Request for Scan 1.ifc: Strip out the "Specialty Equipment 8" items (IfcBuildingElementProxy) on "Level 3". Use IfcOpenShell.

First a look at what the model holds.

```python
import ifcopenshell
import ifcopenshell.util.element

model = ifcopenshell.open("Scan 1.ifc")
print(model.schema)
storey = next(s for s in model.by_type("IfcBuildingStorey") if s.Name == "Level 3")
proxies = [e for e in ifcopenshell.util.element.get_decomposition(storey) if e.is_a("IfcBuildingElementProxy")]
seen = {}
for e in proxies:
    element_type = ifcopenshell.util.element.get_type(e)
    name = element_type.Name if element_type not in (None, e) else None
    seen[name] = seen.get(name, 0) + 1
for name, count in sorted(seen.items(), key=str):
    print(count, "x", name)
```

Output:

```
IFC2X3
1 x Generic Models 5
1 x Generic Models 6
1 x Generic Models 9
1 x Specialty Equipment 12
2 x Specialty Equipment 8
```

```python
import ifcopenshell
import ifcopenshell.api.root
import ifcopenshell.util.element

model = ifcopenshell.open("Scan 1.ifc")

storey = next(s for s in model.by_type("IfcBuildingStorey") if s.Name == "Level 3")
proxies = [e for e in ifcopenshell.util.element.get_decomposition(storey) if e.is_a("IfcBuildingElementProxy")]
targets = [e for e in proxies if (t := ifcopenshell.util.element.get_type(e)) not in (None, e) and t.Name == "Specialty Equipment 8"]

for e in targets:
    ifcopenshell.api.root.remove_product(model, product=e)
print(len(targets), "removed")

model.write("Scan 1_updated.ifc")
```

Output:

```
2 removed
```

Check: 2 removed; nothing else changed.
